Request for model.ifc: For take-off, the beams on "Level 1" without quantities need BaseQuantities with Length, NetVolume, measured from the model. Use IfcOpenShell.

First a look at what the model holds.

```python
import ifcopenshell
import ifcopenshell.util.element
import ifcopenshell.util.unit

model = ifcopenshell.open("model.ifc")
print(model.schema)
for unit_type in ("LENGTHUNIT", "AREAUNIT", "VOLUMEUNIT"):
    print(unit_type, ifcopenshell.util.unit.calculate_unit_scale(model, unit_type))
storey = next(s for s in model.by_type("IfcBuildingStorey") if s.Name == "Level 1")
beams = [e for e in ifcopenshell.util.element.get_decomposition(storey) if e.is_a("IfcBeam")]
for e in sorted(beams, key=lambda e: e.id()):
    print(e.id(), e.is_a(), e.Name, list(ifcopenshell.util.element.get_psets(e, qtos_only=True)), sep=" | ")
```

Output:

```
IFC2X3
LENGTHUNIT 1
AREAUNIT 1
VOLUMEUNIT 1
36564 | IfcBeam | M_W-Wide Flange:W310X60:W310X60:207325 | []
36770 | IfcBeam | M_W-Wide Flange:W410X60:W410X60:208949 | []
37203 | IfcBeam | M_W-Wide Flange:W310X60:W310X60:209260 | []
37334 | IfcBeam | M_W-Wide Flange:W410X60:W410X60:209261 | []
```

```python
import ifcopenshell
import ifcopenshell.api.pset
import ifcopenshell.geom
import ifcopenshell.util.element
import ifcopenshell.util.shape
import ifcopenshell.util.unit

model = ifcopenshell.open("model.ifc")
unit_scale = ifcopenshell.util.unit.calculate_unit_scale(model)
volume_scale = ifcopenshell.util.unit.calculate_unit_scale(model, "VOLUMEUNIT")
settings = ifcopenshell.geom.settings()

storey = next(s for s in model.by_type("IfcBuildingStorey") if s.Name == "Level 1")
beams = [e for e in ifcopenshell.util.element.get_decomposition(storey) if e.is_a("IfcBeam")]

for e in sorted(beams, key=lambda e: e.id()):
    if ifcopenshell.util.element.get_psets(e, qtos_only=True, should_inherit=False):
        continue
    # Geometry comes back in metres, in the element's own axes.
    shape = ifcopenshell.geom.create_shape(settings, e)
    values = {
        "Length": ifcopenshell.util.shape.get_max_xyz(shape.geometry) / unit_scale,
        "NetVolume": ifcopenshell.util.shape.get_volume(shape.geometry) / volume_scale,
    }
    qto = ifcopenshell.api.pset.add_qto(model, product=e, name="BaseQuantities")
    ifcopenshell.api.pset.edit_qto(model, qto=qto, properties=values)
    print(e.id(), {k: round(v, 3) for k, v in values.items()})

model.write("model_v2.ifc")
```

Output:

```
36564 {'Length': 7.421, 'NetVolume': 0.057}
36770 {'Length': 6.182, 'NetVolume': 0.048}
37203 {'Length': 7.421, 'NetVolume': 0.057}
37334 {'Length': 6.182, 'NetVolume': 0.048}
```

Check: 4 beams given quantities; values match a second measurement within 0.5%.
